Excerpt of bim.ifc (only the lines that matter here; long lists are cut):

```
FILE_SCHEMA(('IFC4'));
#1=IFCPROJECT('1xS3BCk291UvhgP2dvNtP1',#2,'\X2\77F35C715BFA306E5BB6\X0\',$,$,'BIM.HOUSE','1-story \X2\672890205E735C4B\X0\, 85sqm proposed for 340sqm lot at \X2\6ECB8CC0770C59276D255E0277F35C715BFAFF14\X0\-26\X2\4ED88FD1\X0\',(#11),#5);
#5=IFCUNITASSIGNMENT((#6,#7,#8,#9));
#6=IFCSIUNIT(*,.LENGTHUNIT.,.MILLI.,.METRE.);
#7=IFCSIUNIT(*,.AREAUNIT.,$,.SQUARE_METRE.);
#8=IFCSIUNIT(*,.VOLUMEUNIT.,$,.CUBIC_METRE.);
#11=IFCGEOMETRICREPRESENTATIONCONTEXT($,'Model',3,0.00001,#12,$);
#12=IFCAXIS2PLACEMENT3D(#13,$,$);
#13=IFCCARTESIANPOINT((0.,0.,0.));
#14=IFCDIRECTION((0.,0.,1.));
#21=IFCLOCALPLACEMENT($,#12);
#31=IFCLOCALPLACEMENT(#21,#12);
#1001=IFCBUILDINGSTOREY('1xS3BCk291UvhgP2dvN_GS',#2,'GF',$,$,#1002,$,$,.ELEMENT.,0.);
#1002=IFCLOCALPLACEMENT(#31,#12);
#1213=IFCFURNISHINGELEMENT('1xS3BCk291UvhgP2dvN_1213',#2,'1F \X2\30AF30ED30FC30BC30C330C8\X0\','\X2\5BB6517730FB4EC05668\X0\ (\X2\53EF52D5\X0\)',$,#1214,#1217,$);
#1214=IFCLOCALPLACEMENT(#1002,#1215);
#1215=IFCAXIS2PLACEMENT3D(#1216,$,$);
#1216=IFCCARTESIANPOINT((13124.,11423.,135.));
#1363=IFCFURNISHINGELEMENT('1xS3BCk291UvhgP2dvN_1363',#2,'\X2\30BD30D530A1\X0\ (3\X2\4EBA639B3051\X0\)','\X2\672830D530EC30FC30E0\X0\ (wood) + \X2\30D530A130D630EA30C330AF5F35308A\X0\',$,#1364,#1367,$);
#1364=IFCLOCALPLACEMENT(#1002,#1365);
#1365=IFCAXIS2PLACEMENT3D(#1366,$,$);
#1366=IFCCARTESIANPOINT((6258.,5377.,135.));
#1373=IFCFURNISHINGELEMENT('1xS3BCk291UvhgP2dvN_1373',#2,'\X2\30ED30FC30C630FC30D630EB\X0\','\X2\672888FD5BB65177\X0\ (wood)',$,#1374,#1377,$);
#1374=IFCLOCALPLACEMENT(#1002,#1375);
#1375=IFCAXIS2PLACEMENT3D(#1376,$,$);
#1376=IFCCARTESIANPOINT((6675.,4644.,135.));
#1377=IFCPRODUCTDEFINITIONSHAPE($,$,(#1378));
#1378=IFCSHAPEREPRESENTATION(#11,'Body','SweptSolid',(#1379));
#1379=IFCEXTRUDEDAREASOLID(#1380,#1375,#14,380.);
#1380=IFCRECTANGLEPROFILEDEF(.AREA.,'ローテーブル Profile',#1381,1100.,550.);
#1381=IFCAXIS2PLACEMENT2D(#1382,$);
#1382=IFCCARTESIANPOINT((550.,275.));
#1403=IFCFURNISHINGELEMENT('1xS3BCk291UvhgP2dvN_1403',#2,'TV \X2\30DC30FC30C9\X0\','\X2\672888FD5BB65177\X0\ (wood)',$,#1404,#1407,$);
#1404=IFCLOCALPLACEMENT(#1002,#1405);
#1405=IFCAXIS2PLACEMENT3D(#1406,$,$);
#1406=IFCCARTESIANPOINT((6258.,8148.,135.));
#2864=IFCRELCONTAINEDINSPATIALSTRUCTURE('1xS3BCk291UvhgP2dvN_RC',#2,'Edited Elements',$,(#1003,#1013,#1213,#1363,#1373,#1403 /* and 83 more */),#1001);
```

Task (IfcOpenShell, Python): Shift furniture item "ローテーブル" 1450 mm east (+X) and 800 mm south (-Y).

```python
import ifcopenshell
import ifcopenshell.api.geometry
import ifcopenshell.util.placement

model = ifcopenshell.open("bim.ifc")

item = model.by_guid("1xS3BCk291UvhgP2dvN_1373")
matrix = ifcopenshell.util.placement.get_local_placement(item.ObjectPlacement)
matrix[0, 3] += 1450.0
matrix[1, 3] -= 800.0
ifcopenshell.api.geometry.edit_object_placement(model, product=item, matrix=matrix, is_si=False)

print(ifcopenshell.util.placement.get_local_placement(item.ObjectPlacement).round(3) + 0.0)

model.write("bim_edited.ifc")
```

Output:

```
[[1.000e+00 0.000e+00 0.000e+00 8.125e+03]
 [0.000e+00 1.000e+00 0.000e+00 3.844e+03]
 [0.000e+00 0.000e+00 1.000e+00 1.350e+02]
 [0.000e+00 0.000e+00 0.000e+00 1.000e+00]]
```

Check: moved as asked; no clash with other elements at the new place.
